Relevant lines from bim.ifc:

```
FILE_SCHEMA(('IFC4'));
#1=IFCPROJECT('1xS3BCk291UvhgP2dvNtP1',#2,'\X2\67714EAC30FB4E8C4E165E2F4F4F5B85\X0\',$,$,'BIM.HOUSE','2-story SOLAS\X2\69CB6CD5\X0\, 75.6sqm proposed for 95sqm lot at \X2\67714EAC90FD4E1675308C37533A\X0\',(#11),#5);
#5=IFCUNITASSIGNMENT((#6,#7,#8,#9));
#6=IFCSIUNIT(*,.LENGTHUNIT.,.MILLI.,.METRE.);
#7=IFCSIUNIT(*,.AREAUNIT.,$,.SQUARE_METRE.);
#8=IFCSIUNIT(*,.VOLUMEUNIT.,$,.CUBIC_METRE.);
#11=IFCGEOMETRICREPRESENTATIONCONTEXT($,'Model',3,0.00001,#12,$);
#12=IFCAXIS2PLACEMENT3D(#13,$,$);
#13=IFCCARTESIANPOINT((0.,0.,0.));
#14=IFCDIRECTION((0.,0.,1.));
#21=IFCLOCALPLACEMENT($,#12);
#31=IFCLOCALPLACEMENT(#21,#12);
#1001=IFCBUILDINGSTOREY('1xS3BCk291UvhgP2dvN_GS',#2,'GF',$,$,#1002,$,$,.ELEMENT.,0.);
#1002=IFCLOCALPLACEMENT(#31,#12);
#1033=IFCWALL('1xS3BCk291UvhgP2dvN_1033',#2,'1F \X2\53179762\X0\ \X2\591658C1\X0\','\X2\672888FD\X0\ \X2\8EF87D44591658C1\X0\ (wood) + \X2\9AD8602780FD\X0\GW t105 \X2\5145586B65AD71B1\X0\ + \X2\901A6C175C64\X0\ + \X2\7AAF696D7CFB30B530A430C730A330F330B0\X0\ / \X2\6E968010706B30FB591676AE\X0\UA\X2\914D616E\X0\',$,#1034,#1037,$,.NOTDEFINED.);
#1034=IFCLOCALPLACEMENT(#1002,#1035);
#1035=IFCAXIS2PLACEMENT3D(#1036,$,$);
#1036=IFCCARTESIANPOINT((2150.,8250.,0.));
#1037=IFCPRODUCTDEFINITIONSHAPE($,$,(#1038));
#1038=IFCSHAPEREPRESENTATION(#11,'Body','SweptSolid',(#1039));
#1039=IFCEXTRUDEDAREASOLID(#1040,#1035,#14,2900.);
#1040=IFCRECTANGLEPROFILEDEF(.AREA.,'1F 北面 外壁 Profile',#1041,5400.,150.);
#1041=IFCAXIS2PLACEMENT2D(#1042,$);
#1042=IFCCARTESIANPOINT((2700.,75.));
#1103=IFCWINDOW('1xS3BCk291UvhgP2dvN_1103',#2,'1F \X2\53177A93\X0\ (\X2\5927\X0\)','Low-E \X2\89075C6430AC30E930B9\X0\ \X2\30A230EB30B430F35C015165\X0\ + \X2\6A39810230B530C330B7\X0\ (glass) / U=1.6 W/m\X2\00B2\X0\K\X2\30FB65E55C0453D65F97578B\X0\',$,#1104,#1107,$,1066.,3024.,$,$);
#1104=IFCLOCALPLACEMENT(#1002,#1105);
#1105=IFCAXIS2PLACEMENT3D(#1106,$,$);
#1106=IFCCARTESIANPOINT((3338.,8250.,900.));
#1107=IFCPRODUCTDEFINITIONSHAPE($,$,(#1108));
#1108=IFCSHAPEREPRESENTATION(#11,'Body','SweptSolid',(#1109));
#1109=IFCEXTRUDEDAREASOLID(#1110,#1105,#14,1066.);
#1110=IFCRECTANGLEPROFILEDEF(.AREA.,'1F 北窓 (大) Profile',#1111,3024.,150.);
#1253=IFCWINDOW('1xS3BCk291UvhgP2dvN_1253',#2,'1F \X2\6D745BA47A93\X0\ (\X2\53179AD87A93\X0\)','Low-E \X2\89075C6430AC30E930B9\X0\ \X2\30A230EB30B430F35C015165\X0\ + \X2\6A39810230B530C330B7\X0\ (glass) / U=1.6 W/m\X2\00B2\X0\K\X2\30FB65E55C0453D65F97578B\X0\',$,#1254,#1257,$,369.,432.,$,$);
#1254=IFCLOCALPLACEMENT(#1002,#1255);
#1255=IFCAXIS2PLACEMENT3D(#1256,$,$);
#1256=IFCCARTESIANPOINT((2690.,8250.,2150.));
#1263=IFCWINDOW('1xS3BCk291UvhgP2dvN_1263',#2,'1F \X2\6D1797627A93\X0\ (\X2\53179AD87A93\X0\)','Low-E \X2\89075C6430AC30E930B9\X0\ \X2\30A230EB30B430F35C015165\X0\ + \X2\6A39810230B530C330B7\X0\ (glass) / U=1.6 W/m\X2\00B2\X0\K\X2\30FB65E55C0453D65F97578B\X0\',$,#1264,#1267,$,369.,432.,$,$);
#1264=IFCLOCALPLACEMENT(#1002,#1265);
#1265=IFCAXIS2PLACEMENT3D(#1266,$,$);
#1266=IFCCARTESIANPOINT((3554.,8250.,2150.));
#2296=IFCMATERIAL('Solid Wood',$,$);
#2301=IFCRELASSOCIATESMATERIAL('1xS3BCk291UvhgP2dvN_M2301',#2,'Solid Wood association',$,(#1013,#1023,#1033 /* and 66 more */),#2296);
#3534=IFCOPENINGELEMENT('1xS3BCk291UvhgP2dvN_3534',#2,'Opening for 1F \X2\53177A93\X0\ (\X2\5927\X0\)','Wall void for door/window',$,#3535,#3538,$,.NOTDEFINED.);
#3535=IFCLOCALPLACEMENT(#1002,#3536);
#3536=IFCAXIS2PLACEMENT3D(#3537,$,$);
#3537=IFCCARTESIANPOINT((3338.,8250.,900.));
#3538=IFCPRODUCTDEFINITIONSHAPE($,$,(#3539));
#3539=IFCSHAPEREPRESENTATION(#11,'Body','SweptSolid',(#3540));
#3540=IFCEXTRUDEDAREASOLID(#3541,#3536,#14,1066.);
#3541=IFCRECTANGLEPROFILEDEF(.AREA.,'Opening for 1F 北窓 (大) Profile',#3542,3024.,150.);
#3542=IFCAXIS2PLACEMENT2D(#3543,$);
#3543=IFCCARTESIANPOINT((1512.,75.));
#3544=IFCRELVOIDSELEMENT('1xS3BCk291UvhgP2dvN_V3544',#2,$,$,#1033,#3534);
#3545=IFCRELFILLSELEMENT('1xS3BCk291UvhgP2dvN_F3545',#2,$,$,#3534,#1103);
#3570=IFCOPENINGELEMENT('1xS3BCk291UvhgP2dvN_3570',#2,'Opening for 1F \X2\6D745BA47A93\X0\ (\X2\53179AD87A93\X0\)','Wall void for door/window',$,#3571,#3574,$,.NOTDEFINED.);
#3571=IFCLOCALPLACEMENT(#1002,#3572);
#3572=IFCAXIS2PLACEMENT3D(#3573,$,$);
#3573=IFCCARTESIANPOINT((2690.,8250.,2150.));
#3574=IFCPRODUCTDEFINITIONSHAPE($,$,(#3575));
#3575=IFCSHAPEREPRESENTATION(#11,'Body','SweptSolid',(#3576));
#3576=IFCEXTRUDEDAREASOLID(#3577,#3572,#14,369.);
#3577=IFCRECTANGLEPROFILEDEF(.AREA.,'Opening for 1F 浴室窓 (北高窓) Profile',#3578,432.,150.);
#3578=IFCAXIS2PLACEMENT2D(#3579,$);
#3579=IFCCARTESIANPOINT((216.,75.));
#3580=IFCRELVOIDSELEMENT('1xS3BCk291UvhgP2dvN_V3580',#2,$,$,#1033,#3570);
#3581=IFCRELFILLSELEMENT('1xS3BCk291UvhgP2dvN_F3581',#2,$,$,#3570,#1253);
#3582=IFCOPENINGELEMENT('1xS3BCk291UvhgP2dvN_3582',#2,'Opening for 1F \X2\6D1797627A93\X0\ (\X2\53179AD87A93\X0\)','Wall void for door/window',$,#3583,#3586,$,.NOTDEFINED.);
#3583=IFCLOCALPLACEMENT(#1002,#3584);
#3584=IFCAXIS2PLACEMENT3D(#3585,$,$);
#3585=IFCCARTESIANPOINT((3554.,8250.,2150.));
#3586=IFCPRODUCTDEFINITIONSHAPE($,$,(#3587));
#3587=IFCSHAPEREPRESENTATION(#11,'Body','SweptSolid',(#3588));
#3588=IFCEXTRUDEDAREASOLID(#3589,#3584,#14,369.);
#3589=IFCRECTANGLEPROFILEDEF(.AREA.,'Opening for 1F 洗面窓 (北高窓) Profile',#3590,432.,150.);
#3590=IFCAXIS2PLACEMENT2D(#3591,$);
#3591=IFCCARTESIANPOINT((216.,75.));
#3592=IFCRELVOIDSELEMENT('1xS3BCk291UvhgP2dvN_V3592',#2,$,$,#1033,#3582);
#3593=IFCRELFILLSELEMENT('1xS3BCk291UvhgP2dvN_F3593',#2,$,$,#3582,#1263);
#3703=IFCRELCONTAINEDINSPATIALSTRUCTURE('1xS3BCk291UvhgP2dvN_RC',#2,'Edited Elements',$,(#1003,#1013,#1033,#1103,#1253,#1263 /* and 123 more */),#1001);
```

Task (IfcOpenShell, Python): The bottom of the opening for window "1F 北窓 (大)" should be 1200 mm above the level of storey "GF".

```python
import numpy as np
import ifcopenshell
import ifcopenshell.api.geometry
import ifcopenshell.geom
import ifcopenshell.util.element
import ifcopenshell.util.placement
import ifcopenshell.util.shape
import ifcopenshell.util.unit

model = ifcopenshell.open("bim.ifc")
unit_scale = ifcopenshell.util.unit.calculate_unit_scale(model)

window = model.by_guid("1xS3BCk291UvhgP2dvN_1103")
opening = window.FillsVoids[0].RelatingOpeningElement
storey = ifcopenshell.util.element.get_container(window, ifc_class="IfcBuildingStorey")
level = ifcopenshell.util.placement.get_local_placement(storey.ObjectPlacement)[2, 3]

# The opening's origin need not be at the sill, so measure its lowest point.
shape = ifcopenshell.geom.create_shape(ifcopenshell.geom.settings(), opening)
bottom = ifcopenshell.util.shape.get_shape_bottom_elevation(shape, shape.geometry) / unit_scale
dz = level + 1.2 / unit_scale - bottom

shift = np.array([0.0, 0.0, dz])
# The window is not placed relative to its opening, so move both.
for product in (opening, window):
    matrix = ifcopenshell.util.placement.get_local_placement(product.ObjectPlacement)
    matrix[:3, 3] += shift
    ifcopenshell.api.geometry.edit_object_placement(model, product=product, matrix=matrix, is_si=False)

print(f"moved by {dz * unit_scale:+.3f} m")

model.write("bim_v2.ifc")
```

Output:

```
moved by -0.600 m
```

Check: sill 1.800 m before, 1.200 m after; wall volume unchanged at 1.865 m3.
